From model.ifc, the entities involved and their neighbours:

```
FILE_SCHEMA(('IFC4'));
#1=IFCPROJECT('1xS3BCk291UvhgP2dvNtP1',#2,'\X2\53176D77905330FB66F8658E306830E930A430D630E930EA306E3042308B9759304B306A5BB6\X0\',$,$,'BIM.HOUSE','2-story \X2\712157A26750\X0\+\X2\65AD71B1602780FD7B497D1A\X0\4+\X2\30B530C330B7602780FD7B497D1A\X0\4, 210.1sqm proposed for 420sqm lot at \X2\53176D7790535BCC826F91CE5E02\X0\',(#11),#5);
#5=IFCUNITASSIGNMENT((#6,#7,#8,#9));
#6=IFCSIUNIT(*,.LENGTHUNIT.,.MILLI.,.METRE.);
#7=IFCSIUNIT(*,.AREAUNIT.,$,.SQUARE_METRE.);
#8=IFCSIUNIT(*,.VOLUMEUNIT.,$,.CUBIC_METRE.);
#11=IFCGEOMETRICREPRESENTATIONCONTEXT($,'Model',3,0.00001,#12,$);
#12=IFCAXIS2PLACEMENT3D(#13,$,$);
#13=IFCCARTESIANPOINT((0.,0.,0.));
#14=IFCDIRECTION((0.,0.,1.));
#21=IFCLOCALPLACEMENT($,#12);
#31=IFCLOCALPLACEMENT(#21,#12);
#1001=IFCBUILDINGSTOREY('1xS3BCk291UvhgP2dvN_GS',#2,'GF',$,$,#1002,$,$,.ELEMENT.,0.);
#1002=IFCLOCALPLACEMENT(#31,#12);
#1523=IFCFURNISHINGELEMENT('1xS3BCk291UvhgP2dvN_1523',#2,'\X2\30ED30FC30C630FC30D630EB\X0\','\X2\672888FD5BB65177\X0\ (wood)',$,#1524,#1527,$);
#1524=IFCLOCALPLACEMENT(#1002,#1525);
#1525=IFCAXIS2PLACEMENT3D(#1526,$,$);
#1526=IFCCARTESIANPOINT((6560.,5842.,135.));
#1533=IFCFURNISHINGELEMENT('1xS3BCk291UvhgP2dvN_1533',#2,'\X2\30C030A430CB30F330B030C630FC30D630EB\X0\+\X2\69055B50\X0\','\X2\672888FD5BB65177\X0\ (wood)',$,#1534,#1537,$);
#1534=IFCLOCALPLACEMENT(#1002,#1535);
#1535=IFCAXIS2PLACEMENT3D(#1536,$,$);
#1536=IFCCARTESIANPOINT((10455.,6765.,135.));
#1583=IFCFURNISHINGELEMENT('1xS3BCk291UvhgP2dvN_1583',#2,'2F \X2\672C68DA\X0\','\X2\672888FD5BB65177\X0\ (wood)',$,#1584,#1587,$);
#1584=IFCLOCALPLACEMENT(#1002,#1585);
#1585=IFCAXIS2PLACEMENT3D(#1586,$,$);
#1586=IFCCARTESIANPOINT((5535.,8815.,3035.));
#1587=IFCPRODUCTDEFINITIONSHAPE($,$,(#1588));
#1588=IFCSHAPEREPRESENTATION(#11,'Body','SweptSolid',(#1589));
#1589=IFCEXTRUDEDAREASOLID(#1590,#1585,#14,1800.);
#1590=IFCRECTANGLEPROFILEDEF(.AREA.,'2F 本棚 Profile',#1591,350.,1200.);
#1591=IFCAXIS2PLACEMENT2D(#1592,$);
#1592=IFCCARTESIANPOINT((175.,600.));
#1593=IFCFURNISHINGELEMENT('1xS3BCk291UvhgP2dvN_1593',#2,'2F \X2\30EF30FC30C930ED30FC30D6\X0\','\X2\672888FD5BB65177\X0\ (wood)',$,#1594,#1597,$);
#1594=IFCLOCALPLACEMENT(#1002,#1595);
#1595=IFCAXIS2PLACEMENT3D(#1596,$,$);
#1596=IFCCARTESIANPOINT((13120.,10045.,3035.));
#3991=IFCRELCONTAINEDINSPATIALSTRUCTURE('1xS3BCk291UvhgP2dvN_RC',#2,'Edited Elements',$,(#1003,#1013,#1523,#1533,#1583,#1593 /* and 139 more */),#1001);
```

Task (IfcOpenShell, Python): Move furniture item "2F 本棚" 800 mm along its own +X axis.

```python
import ifcopenshell
import ifcopenshell.api.geometry
import ifcopenshell.util.placement

model = ifcopenshell.open("model.ifc")

item = model.by_guid("1xS3BCk291UvhgP2dvN_1583")
matrix = ifcopenshell.util.placement.get_local_placement(item.ObjectPlacement)
matrix[:3, 3] += matrix[:3, 0] * 800.0
ifcopenshell.api.geometry.edit_object_placement(model, product=item, matrix=matrix, is_si=False)

print(ifcopenshell.util.placement.get_local_placement(item.ObjectPlacement).round(3) + 0.0)

model.write("model_edited.ifc")
```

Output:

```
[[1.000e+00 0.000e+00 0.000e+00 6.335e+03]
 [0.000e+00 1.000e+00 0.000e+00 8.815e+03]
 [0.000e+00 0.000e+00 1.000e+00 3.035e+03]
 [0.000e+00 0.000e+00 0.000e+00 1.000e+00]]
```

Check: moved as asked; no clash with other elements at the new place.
